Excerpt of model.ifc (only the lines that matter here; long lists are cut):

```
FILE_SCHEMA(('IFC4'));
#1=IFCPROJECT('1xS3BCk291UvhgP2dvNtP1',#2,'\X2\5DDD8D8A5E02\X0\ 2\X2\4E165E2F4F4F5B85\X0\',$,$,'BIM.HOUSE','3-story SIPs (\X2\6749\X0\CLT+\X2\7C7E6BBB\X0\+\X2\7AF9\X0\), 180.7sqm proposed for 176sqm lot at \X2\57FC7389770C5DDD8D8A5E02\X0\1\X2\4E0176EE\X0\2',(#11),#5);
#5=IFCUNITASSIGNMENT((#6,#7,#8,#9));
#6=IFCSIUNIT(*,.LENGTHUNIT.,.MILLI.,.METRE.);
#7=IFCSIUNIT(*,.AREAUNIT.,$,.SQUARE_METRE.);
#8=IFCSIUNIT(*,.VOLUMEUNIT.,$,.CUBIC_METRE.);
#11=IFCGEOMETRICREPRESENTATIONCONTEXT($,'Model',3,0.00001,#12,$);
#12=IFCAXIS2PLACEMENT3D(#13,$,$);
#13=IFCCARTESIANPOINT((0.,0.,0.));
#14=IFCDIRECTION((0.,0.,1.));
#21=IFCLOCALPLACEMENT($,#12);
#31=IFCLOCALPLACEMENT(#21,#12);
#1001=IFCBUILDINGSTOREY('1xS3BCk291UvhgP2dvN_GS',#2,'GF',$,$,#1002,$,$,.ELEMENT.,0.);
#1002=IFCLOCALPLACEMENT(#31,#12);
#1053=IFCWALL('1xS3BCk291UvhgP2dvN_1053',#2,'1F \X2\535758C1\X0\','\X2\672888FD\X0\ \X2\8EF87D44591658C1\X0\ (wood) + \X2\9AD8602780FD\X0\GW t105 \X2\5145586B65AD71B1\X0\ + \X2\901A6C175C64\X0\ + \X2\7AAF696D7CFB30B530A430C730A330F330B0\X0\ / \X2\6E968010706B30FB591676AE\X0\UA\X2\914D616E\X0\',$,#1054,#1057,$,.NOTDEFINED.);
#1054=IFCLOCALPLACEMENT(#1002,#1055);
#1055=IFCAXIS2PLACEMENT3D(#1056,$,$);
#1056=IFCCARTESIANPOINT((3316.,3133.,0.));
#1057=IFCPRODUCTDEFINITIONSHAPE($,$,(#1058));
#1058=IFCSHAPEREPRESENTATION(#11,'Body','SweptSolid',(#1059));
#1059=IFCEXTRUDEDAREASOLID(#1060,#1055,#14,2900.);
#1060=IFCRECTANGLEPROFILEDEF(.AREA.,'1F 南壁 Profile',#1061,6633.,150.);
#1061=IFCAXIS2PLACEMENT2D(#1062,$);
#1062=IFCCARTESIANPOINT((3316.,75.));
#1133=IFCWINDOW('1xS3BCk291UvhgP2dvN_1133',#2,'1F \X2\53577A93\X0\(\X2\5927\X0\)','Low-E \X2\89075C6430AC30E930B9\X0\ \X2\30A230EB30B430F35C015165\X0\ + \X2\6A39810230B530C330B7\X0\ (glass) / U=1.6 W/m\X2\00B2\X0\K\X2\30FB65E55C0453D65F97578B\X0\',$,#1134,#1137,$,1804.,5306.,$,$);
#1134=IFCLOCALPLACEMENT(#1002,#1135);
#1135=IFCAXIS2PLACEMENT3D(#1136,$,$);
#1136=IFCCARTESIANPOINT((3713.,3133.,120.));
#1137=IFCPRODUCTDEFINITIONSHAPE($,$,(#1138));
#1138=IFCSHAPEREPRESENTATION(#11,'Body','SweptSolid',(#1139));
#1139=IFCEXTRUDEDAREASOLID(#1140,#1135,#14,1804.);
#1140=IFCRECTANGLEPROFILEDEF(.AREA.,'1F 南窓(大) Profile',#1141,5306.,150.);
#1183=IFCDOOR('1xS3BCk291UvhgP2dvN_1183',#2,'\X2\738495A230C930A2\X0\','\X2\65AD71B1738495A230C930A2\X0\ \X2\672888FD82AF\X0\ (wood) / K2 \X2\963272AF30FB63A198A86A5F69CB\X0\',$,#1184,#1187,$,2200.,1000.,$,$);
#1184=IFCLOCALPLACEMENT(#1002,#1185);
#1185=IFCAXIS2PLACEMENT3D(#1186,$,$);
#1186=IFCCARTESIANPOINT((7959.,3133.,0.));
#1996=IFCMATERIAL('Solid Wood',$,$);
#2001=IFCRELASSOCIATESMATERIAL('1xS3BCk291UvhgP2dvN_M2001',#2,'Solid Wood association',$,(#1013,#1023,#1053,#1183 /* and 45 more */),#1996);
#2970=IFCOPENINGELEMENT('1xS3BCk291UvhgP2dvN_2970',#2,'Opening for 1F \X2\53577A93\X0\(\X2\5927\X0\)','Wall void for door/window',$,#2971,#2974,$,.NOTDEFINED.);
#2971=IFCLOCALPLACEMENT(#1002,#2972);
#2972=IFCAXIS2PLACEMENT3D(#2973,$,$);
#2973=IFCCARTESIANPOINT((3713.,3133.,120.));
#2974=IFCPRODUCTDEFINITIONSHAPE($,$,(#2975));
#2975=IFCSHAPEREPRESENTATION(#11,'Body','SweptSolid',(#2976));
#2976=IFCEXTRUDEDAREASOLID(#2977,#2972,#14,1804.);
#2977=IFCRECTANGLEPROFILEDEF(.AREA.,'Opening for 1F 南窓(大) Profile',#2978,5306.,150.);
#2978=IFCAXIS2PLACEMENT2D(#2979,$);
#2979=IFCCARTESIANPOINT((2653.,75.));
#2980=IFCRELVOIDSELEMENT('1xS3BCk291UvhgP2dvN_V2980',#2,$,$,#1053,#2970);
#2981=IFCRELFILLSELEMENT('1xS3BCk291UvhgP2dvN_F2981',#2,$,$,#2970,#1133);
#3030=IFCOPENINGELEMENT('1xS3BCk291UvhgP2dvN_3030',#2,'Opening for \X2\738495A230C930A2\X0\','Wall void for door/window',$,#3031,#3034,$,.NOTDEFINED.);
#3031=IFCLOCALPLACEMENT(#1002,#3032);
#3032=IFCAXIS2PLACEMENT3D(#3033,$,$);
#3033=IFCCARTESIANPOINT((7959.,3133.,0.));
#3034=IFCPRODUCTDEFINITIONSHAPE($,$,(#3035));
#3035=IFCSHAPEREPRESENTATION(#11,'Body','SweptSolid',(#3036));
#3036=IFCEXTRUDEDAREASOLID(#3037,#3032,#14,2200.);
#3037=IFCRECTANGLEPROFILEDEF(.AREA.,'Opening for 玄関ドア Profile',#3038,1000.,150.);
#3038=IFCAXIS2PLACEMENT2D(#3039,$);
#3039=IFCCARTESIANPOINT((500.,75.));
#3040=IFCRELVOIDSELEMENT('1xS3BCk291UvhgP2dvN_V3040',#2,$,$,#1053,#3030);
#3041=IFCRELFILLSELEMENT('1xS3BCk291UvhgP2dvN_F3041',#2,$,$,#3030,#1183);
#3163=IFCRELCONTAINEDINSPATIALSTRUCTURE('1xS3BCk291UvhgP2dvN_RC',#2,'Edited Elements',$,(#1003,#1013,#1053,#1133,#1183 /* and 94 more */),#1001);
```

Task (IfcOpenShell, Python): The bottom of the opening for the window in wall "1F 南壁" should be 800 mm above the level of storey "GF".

```python
import numpy as np
import ifcopenshell
import ifcopenshell.api.geometry
import ifcopenshell.geom
import ifcopenshell.util.element
import ifcopenshell.util.placement
import ifcopenshell.util.shape
import ifcopenshell.util.unit

model = ifcopenshell.open("model.ifc")
unit_scale = ifcopenshell.util.unit.calculate_unit_scale(model)

window = model.by_guid("1xS3BCk291UvhgP2dvN_1133")
opening = window.FillsVoids[0].RelatingOpeningElement
storey = ifcopenshell.util.element.get_container(window, ifc_class="IfcBuildingStorey")
level = ifcopenshell.util.placement.get_local_placement(storey.ObjectPlacement)[2, 3]

# The opening's origin need not be at the sill, so measure its lowest point.
shape = ifcopenshell.geom.create_shape(ifcopenshell.geom.settings(), opening)
bottom = ifcopenshell.util.shape.get_shape_bottom_elevation(shape, shape.geometry) / unit_scale
dz = level + 800.0 - bottom

shift = np.array([0.0, 0.0, dz])
# The window is not placed relative to its opening, so move both.
for product in (opening, window):
    matrix = ifcopenshell.util.placement.get_local_placement(product.ObjectPlacement)
    matrix[:3, 3] += shift
    ifcopenshell.api.geometry.edit_object_placement(model, product=product, matrix=matrix, is_si=False)

print(f"moved by {dz * unit_scale:+.3f} m")

model.write("model_v2.ifc")
```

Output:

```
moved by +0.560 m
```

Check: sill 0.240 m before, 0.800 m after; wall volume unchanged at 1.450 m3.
